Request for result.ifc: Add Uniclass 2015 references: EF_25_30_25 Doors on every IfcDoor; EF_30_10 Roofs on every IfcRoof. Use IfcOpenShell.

First a look at what the model holds.

```python
import ifcopenshell

model = ifcopenshell.open("result.ifc")
print(model.schema)
print("classifications:", [c.Name for c in model.by_type("IfcClassification")])
for ifc_class in ("IfcDoor", "IfcRoof", "IfcStair", "IfcWall", "IfcWindow"):
    print(ifc_class, len(model.by_type(ifc_class)))
```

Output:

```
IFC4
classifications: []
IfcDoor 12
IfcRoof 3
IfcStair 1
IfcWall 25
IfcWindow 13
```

```python
import ifcopenshell
import ifcopenshell.api.classification

model = ifcopenshell.open("result.ifc")

system = ifcopenshell.api.classification.add_classification(model, classification="Uniclass 2015")

codes = {
    "IfcDoor": ("EF_25_30_25", "Doors"),
    "IfcRoof": ("EF_30_10", "Roofs"),
}
for ifc_class, (code, name) in codes.items():
    products = model.by_type(ifc_class)
    ifcopenshell.api.classification.add_reference(
        model, products=products, classification=system, identification=code, name=name
    )
    print(code, len(products))

model.write("result_edited.ifc")
```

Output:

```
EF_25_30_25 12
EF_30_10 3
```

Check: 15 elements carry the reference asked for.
